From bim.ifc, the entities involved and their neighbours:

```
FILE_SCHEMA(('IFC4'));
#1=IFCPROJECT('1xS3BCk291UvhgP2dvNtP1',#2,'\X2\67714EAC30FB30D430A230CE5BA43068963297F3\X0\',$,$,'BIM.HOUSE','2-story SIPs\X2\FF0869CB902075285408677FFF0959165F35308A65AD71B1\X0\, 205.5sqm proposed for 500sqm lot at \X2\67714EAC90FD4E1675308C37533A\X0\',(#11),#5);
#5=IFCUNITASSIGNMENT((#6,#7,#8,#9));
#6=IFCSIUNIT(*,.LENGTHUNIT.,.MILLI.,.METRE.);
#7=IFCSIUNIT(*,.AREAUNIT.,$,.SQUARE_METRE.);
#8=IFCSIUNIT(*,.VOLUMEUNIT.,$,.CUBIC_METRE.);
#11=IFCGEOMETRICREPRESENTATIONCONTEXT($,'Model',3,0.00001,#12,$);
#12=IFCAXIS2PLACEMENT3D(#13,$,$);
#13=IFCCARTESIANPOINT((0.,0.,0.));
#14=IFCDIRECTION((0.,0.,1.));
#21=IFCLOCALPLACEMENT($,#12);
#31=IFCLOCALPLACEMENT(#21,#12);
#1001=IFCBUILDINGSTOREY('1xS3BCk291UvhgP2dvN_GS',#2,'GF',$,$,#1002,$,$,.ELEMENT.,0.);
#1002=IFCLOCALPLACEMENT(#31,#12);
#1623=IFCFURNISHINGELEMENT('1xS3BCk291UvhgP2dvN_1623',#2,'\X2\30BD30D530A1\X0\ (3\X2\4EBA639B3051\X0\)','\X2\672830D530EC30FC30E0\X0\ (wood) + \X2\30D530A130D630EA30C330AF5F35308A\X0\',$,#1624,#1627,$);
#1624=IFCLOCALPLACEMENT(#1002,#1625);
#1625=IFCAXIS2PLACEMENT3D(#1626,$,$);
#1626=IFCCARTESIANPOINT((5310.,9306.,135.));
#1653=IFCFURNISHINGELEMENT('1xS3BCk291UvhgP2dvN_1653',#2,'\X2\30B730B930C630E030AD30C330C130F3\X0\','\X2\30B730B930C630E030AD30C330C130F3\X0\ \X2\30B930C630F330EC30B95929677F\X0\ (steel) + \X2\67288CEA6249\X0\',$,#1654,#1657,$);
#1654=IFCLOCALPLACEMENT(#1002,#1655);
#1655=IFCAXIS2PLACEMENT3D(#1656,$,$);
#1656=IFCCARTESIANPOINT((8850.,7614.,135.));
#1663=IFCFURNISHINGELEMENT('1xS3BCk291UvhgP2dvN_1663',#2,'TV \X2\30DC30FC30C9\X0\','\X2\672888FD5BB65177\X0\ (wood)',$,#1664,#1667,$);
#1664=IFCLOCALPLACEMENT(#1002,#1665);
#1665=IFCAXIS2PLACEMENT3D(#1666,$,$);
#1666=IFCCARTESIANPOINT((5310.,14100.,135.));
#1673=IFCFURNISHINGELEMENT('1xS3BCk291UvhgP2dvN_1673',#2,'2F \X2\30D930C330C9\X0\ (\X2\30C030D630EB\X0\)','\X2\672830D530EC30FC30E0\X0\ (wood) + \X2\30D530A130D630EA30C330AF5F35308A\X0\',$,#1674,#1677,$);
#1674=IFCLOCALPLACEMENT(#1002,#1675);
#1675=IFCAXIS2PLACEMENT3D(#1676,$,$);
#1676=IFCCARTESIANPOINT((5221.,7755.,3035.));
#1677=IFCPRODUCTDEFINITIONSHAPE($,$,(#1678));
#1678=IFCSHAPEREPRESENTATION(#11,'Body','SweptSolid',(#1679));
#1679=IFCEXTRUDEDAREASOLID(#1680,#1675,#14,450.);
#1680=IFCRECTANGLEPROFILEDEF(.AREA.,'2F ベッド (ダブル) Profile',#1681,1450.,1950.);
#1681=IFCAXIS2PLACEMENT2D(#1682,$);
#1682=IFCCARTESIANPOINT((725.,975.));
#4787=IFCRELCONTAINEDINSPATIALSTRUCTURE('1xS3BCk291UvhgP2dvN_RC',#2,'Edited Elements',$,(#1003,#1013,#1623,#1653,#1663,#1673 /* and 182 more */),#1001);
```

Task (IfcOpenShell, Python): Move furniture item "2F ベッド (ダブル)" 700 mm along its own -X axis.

```python
import ifcopenshell
import ifcopenshell.api.geometry
import ifcopenshell.util.placement
import ifcopenshell.util.unit

model = ifcopenshell.open("bim.ifc")
unit_scale = ifcopenshell.util.unit.calculate_unit_scale(model)

item = model.by_guid("1xS3BCk291UvhgP2dvN_1673")
matrix = ifcopenshell.util.placement.get_local_placement(item.ObjectPlacement)
matrix[:3, 3] -= matrix[:3, 0] * 0.7 / unit_scale
ifcopenshell.api.geometry.edit_object_placement(model, product=item, matrix=matrix, is_si=False)

print(ifcopenshell.util.placement.get_local_placement(item.ObjectPlacement).round(3) + 0.0)

model.write("bim_rev.ifc")
```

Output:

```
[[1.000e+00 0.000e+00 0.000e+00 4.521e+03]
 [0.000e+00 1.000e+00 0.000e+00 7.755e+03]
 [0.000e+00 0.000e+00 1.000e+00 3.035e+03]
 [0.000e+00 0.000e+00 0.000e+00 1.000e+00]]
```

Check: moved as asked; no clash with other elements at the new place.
